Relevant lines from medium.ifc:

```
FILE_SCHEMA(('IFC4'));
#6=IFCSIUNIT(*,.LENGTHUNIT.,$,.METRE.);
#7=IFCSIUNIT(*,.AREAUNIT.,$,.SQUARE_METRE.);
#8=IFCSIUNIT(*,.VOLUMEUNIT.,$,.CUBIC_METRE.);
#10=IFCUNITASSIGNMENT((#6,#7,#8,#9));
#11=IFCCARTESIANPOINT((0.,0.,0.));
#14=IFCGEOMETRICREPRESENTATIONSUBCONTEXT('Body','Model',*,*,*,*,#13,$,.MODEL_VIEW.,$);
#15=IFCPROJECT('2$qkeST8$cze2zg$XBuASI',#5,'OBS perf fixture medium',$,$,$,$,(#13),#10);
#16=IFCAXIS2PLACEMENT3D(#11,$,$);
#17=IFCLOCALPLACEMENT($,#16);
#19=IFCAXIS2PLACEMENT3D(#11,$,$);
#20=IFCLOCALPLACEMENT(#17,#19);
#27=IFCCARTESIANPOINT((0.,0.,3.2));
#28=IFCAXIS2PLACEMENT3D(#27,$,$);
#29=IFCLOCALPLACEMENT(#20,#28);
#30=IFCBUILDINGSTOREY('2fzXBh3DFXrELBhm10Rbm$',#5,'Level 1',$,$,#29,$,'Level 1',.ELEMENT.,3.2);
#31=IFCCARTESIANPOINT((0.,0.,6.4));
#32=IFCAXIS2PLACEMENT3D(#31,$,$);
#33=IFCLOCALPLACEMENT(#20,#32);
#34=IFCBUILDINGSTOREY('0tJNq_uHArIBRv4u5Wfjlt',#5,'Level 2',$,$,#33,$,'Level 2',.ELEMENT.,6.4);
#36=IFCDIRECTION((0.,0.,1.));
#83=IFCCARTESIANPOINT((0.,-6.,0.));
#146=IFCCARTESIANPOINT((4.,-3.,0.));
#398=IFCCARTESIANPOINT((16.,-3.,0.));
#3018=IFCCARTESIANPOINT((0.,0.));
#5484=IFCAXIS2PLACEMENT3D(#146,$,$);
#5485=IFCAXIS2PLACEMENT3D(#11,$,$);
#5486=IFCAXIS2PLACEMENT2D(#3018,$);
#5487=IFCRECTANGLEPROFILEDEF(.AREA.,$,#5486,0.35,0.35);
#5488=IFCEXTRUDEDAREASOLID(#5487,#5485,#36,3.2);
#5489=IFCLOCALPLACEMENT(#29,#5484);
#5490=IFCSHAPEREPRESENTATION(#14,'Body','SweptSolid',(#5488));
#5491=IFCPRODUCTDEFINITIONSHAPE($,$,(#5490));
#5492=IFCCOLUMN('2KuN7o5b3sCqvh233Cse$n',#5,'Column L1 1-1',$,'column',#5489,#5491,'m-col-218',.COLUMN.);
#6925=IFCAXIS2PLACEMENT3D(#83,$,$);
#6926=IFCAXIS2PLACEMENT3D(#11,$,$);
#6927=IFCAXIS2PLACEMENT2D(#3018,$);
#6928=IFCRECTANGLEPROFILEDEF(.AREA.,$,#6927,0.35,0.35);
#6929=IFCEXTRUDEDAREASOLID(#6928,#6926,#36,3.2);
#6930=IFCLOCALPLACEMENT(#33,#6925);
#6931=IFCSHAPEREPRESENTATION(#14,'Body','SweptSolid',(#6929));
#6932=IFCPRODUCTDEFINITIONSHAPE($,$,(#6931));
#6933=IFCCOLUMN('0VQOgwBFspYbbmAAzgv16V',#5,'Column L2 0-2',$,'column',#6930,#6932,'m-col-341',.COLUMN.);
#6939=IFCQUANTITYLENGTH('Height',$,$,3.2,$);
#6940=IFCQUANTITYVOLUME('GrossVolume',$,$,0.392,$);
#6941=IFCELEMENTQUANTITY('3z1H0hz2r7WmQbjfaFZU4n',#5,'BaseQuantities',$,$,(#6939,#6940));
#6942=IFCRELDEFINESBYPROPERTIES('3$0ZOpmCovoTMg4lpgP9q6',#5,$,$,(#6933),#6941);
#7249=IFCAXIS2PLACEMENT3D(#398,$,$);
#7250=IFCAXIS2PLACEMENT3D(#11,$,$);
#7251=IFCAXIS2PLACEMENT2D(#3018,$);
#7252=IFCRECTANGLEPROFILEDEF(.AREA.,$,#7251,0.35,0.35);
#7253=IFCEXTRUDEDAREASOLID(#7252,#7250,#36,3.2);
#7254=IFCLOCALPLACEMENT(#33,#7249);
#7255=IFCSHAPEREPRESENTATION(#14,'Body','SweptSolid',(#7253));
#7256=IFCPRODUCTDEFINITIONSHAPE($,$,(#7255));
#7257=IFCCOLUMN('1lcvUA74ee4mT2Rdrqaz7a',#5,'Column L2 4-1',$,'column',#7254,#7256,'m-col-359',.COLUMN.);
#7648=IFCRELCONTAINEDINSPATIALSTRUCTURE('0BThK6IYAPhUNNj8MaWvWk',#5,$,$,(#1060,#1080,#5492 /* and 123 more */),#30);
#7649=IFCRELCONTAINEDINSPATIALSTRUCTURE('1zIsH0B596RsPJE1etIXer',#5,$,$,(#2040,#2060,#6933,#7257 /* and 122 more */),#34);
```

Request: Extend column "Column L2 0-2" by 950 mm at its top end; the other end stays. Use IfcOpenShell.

```python
import ifcopenshell
import ifcopenshell.api.pset
import ifcopenshell.util.element
import ifcopenshell.util.representation
import ifcopenshell.util.unit

model = ifcopenshell.open("medium.ifc")
unit_scale = ifcopenshell.util.unit.calculate_unit_scale(model)

member = model.by_id(6933)
change = 0.95 / unit_scale

# The extrusion runs towards the end named, so only its depth changes.
body = ifcopenshell.util.representation.get_representation(member, "Model", "Body")
solid = body.Items[0]
old_length = solid.Depth
solid.Depth += change

# Update the stored length and volume.
qto = model.by_id(ifcopenshell.util.element.get_pset(member, "BaseQuantities", should_inherit=False)["id"])
ifcopenshell.api.pset.edit_qto(model, qto=qto, properties={
    "Height": solid.Depth,
    "GrossVolume": ifcopenshell.util.element.get_pset(member, "BaseQuantities", "GrossVolume") * solid.Depth / old_length,
})

print(f"length {old_length:g} -> {solid.Depth:g}")

model.write("medium_updated.ifc")
```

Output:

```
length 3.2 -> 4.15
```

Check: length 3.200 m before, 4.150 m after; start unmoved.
